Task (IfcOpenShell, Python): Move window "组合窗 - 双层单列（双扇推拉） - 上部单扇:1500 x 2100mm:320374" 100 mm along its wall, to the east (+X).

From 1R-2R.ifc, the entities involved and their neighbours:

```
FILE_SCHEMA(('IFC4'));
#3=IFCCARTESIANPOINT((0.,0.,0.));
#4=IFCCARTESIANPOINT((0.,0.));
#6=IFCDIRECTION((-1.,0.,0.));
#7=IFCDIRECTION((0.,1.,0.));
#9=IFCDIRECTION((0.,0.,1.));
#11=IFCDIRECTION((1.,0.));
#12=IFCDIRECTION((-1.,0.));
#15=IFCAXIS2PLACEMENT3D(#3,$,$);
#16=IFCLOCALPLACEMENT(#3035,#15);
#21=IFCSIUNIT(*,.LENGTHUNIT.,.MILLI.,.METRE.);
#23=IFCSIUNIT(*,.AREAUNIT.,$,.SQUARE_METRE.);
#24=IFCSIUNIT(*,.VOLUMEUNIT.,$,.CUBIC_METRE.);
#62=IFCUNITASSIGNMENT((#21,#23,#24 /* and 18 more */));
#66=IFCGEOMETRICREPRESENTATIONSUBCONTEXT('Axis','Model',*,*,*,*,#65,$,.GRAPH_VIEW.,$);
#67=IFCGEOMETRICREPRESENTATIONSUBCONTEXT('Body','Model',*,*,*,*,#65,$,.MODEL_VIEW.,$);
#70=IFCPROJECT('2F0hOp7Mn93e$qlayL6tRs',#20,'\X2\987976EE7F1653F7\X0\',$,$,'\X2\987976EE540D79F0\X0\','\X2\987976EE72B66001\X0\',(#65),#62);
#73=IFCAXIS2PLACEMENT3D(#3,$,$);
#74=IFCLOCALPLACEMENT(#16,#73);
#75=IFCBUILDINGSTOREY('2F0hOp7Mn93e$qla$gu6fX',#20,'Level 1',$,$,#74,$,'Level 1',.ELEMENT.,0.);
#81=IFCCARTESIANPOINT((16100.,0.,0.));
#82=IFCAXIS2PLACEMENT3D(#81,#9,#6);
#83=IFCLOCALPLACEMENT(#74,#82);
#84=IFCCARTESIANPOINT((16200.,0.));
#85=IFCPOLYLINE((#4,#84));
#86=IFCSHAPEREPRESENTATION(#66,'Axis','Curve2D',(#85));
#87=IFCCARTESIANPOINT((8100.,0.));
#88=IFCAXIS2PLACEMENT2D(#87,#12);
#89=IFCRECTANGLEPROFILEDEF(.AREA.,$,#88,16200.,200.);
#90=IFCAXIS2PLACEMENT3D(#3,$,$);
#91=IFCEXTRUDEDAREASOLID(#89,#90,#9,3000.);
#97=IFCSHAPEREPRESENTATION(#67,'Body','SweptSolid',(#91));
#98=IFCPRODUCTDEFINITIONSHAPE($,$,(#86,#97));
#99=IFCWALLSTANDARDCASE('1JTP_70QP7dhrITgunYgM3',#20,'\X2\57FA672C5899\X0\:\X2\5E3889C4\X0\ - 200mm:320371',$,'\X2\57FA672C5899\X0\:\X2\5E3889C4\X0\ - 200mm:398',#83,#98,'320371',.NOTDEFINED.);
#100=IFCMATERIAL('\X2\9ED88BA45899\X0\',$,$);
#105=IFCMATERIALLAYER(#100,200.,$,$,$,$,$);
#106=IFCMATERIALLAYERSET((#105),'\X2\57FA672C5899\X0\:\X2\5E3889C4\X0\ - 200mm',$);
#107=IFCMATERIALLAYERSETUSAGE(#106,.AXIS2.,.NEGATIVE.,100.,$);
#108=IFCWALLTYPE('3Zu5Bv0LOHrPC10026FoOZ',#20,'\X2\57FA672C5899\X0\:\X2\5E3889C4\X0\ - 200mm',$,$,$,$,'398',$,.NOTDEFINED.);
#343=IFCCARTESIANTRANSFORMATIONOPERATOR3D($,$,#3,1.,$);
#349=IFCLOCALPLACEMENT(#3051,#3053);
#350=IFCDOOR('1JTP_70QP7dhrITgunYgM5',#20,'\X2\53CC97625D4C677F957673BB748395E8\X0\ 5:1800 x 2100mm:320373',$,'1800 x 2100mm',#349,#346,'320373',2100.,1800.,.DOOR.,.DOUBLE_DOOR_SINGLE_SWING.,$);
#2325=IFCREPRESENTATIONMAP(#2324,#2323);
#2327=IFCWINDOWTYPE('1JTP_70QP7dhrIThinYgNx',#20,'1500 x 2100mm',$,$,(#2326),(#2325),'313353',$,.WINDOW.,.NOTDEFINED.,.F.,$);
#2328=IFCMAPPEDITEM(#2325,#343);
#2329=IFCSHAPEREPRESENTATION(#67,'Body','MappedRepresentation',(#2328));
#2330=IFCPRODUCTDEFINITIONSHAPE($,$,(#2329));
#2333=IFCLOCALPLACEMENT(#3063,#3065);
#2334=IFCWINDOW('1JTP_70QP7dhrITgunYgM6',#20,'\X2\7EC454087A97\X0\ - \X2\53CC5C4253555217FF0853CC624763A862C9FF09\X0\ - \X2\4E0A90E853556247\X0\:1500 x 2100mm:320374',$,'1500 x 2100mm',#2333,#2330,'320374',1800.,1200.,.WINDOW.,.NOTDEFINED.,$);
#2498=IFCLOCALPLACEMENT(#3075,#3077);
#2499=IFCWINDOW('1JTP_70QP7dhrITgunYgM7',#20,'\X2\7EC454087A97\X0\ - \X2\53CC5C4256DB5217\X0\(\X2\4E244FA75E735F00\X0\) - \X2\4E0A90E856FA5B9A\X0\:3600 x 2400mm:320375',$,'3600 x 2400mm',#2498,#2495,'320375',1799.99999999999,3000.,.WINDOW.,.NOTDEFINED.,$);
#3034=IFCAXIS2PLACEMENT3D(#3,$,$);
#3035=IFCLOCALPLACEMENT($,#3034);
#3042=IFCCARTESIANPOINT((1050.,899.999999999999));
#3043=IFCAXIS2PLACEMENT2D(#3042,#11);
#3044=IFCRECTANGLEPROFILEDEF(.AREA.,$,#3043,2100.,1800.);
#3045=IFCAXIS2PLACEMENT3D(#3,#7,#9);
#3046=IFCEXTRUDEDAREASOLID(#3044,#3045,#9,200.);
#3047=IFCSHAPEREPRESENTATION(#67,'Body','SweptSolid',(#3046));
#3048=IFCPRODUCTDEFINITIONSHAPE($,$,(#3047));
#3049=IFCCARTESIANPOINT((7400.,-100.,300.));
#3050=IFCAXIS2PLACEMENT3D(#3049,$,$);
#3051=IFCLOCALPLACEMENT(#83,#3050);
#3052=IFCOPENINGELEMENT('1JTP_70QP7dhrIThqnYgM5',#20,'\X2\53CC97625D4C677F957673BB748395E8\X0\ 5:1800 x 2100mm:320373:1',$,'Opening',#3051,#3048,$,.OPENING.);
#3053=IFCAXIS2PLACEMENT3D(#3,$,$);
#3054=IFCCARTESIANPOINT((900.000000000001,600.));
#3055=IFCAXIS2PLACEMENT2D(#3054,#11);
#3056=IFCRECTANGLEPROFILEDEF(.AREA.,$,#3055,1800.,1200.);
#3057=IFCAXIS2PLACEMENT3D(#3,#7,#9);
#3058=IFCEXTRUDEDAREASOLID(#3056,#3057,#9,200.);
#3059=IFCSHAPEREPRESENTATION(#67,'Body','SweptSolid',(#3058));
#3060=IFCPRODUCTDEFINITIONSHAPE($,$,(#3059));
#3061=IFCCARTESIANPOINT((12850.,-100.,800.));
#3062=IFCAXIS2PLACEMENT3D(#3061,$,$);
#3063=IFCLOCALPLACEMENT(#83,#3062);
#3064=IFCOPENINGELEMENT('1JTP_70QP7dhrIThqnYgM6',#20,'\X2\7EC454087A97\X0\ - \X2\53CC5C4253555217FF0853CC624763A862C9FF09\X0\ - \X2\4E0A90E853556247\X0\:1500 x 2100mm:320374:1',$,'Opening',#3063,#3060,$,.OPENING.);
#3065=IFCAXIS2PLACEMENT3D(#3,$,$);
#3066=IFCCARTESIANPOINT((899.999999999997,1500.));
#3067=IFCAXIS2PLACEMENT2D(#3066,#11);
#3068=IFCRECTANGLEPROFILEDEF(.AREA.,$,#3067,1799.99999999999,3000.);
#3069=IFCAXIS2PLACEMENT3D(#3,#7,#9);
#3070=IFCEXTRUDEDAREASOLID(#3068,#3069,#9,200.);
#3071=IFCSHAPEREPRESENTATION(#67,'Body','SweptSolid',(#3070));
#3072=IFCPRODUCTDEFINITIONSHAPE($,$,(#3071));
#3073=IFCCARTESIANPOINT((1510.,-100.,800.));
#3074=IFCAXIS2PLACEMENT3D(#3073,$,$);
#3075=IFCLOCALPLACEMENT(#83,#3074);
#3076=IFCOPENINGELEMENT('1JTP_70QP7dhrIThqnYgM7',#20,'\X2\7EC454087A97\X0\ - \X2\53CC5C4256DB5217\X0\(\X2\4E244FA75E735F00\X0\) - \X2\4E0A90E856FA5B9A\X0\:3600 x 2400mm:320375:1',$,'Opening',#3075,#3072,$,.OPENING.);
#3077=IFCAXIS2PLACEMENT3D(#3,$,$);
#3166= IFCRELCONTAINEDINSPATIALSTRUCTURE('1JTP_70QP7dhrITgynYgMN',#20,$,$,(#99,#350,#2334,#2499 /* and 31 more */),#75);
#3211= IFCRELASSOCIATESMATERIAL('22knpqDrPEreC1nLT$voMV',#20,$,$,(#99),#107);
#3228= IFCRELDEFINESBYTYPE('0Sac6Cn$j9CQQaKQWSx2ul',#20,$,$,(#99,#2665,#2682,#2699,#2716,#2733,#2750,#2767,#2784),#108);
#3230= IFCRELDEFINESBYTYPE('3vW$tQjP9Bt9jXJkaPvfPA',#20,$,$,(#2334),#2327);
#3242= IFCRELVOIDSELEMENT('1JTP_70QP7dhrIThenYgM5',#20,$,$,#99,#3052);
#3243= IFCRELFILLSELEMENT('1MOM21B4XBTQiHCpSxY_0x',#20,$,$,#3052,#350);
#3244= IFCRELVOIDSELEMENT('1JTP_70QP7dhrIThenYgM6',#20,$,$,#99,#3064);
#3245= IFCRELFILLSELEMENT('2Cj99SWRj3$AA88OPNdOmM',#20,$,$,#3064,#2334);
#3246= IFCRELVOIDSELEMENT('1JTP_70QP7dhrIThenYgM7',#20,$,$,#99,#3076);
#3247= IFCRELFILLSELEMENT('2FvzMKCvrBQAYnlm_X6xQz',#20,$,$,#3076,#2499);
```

```python
import ifcopenshell
import ifcopenshell.api.geometry
import ifcopenshell.util.placement
import ifcopenshell.util.unit

model = ifcopenshell.open("1R-2R.ifc")
unit_scale = ifcopenshell.util.unit.calculate_unit_scale(model)

window = model.by_guid("1JTP_70QP7dhrITgunYgM6")
opening = window.FillsVoids[0].RelatingOpeningElement
wall = opening.VoidsElements[0].RelatingBuildingElement

wall_matrix = ifcopenshell.util.placement.get_local_placement(wall.ObjectPlacement)
shift = wall_matrix[:3, 0] * -0.1 / unit_scale
before = ifcopenshell.util.placement.get_local_placement(window.ObjectPlacement)[:3, 3].copy()

# The window is placed relative to its opening, so it follows when the opening moves.
matrix = ifcopenshell.util.placement.get_local_placement(opening.ObjectPlacement)
matrix[:3, 3] += shift
ifcopenshell.api.geometry.edit_object_placement(
    model, product=opening, matrix=matrix, is_si=False, should_transform_children=True
)

after = ifcopenshell.util.placement.get_local_placement(window.ObjectPlacement)[:3, 3]
print("window moved by", (after - before).round(3) + 0.0)

model.write("1R-2R_updated.ifc")
```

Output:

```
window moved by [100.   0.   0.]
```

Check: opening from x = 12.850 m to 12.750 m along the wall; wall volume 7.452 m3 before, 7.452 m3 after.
